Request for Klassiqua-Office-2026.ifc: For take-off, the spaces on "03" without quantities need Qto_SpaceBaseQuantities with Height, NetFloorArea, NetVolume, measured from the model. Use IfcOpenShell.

First a look at what the model holds.

```python
import ifcopenshell
import ifcopenshell.util.element
import ifcopenshell.util.unit

model = ifcopenshell.open("Klassiqua-Office-2026.ifc")
print(model.schema)
for unit_type in ("LENGTHUNIT", "AREAUNIT", "VOLUMEUNIT"):
    print(unit_type, ifcopenshell.util.unit.calculate_unit_scale(model, unit_type))
storey = next(s for s in model.by_type("IfcBuildingStorey") if s.Name == "03")
spaces = [e for e in ifcopenshell.util.element.get_decomposition(storey) if e.is_a("IfcSpace")]
for e in sorted(spaces, key=lambda e: e.id()):
    print(e.id(), e.is_a(), e.Name, list(ifcopenshell.util.element.get_psets(e, qtos_only=True)), sep=" | ")
```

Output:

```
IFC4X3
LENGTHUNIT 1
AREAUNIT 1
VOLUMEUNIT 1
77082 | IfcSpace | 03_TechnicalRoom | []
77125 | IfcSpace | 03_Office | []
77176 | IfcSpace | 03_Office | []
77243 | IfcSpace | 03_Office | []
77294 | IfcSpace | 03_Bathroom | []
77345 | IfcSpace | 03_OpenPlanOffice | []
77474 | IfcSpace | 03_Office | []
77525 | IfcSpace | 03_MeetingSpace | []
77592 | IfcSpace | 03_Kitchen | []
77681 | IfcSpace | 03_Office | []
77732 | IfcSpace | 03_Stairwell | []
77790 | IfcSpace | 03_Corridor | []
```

```python
import ifcopenshell
import ifcopenshell.api.pset
import ifcopenshell.geom
import ifcopenshell.util.element
import ifcopenshell.util.shape
import ifcopenshell.util.unit

model = ifcopenshell.open("Klassiqua-Office-2026.ifc")
unit_scale = ifcopenshell.util.unit.calculate_unit_scale(model)
area_scale = ifcopenshell.util.unit.calculate_unit_scale(model, "AREAUNIT")
volume_scale = ifcopenshell.util.unit.calculate_unit_scale(model, "VOLUMEUNIT")
settings = ifcopenshell.geom.settings()

storey = next(s for s in model.by_type("IfcBuildingStorey") if s.Name == "03")
spaces = [e for e in ifcopenshell.util.element.get_decomposition(storey) if e.is_a("IfcSpace")]

for e in sorted(spaces, key=lambda e: e.id()):
    if ifcopenshell.util.element.get_psets(e, qtos_only=True, should_inherit=False):
        continue
    # Geometry comes back in metres, in the element's own axes.
    shape = ifcopenshell.geom.create_shape(settings, e)
    values = {
        "Height": ifcopenshell.util.shape.get_z(shape.geometry) / unit_scale,
        "NetFloorArea": ifcopenshell.util.shape.get_footprint_area(shape.geometry) / area_scale,
        "NetVolume": ifcopenshell.util.shape.get_volume(shape.geometry) / volume_scale,
    }
    qto = ifcopenshell.api.pset.add_qto(model, product=e, name="Qto_SpaceBaseQuantities")
    ifcopenshell.api.pset.edit_qto(model, qto=qto, properties=values)
    print(e.id(), {k: round(v, 3) for k, v in values.items()})

model.write("Klassiqua-Office-2026-out.ifc")
```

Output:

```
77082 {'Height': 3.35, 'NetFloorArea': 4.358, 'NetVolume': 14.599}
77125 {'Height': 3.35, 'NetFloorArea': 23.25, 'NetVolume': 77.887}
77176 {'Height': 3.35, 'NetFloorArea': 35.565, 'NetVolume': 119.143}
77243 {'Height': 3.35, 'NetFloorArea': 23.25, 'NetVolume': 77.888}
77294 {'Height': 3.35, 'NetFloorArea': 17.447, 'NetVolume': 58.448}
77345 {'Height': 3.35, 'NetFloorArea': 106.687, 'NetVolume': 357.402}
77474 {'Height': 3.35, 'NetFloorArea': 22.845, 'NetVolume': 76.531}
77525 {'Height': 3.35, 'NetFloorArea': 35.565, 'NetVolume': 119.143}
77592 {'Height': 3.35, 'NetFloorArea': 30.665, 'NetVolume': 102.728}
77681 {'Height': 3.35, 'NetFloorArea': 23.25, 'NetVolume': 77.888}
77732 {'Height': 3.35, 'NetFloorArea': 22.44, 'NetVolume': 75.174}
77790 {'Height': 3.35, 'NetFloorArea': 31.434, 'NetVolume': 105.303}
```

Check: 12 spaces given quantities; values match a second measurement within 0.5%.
